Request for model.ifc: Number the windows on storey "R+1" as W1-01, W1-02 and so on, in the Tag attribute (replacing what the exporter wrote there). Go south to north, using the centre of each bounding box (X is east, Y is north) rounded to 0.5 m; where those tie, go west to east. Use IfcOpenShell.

First a look at what the model holds.

```python
import ifcopenshell
import ifcopenshell.util.element
import ifcopenshell.util.placement

model = ifcopenshell.open("model.ifc")
print(model.schema)
storey = next(s for s in model.by_type("IfcBuildingStorey") if s.Name == "R+1")
windows = [e for e in ifcopenshell.util.element.get_decomposition(storey) if e.is_a("IfcWindow")]
for e in sorted(windows, key=lambda e: e.id()):
    origin = ifcopenshell.util.placement.get_local_placement(e.ObjectPlacement)[:3, 3]
    print(e.id(), e.Tag, e.Name, origin.round(2) + 0.0, sep=" | ")
```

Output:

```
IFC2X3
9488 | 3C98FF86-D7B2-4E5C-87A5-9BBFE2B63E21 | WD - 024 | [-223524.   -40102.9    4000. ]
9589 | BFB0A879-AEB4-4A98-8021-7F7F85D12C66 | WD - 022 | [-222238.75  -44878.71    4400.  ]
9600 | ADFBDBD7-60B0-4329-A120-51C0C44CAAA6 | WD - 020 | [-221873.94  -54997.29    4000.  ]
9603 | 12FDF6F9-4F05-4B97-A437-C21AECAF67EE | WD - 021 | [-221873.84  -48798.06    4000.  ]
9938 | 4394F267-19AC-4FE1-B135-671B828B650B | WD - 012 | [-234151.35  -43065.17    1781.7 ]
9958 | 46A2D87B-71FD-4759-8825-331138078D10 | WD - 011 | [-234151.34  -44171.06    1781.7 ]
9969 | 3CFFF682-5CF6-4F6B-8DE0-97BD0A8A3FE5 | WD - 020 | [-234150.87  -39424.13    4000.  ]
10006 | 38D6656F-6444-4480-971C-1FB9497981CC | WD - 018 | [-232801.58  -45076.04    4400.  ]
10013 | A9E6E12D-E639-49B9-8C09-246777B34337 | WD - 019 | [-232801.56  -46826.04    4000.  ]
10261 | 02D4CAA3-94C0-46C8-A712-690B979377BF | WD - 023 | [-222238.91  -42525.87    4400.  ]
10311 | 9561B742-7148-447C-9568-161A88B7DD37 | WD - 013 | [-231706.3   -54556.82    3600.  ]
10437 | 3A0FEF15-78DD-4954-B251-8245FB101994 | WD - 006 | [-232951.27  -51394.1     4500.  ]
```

```python
import ifcopenshell
import ifcopenshell.geom
import ifcopenshell.util.element
import ifcopenshell.util.shape

model = ifcopenshell.open("model.ifc")
settings = ifcopenshell.geom.settings()
settings.set("use-world-coords", True)


def centre(element):
    shape = ifcopenshell.geom.create_shape(settings, element)
    return ifcopenshell.util.shape.get_bbox_centroid(shape.geometry)


storey = next(s for s in model.by_type("IfcBuildingStorey") if s.Name == "R+1")
windows = [e for e in ifcopenshell.util.element.get_decomposition(storey) if e.is_a("IfcWindow")]

# Insertion points can sit at a corner or the storey origin, so sort by the geometry (in metres).
centres = {e: centre(e) for e in windows}
windows.sort(key=lambda e: (round(centres[e][1] / 0.5), centres[e][0]))

for i, e in enumerate(windows, start=1):
    number = f"W1-{i:02d}"
    e.Tag = number
    print(e.id(), number)

model.write("model_rev.ifc")
```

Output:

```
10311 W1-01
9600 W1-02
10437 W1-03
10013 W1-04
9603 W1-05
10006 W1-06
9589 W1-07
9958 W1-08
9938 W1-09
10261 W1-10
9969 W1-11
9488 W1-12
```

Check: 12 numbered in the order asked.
